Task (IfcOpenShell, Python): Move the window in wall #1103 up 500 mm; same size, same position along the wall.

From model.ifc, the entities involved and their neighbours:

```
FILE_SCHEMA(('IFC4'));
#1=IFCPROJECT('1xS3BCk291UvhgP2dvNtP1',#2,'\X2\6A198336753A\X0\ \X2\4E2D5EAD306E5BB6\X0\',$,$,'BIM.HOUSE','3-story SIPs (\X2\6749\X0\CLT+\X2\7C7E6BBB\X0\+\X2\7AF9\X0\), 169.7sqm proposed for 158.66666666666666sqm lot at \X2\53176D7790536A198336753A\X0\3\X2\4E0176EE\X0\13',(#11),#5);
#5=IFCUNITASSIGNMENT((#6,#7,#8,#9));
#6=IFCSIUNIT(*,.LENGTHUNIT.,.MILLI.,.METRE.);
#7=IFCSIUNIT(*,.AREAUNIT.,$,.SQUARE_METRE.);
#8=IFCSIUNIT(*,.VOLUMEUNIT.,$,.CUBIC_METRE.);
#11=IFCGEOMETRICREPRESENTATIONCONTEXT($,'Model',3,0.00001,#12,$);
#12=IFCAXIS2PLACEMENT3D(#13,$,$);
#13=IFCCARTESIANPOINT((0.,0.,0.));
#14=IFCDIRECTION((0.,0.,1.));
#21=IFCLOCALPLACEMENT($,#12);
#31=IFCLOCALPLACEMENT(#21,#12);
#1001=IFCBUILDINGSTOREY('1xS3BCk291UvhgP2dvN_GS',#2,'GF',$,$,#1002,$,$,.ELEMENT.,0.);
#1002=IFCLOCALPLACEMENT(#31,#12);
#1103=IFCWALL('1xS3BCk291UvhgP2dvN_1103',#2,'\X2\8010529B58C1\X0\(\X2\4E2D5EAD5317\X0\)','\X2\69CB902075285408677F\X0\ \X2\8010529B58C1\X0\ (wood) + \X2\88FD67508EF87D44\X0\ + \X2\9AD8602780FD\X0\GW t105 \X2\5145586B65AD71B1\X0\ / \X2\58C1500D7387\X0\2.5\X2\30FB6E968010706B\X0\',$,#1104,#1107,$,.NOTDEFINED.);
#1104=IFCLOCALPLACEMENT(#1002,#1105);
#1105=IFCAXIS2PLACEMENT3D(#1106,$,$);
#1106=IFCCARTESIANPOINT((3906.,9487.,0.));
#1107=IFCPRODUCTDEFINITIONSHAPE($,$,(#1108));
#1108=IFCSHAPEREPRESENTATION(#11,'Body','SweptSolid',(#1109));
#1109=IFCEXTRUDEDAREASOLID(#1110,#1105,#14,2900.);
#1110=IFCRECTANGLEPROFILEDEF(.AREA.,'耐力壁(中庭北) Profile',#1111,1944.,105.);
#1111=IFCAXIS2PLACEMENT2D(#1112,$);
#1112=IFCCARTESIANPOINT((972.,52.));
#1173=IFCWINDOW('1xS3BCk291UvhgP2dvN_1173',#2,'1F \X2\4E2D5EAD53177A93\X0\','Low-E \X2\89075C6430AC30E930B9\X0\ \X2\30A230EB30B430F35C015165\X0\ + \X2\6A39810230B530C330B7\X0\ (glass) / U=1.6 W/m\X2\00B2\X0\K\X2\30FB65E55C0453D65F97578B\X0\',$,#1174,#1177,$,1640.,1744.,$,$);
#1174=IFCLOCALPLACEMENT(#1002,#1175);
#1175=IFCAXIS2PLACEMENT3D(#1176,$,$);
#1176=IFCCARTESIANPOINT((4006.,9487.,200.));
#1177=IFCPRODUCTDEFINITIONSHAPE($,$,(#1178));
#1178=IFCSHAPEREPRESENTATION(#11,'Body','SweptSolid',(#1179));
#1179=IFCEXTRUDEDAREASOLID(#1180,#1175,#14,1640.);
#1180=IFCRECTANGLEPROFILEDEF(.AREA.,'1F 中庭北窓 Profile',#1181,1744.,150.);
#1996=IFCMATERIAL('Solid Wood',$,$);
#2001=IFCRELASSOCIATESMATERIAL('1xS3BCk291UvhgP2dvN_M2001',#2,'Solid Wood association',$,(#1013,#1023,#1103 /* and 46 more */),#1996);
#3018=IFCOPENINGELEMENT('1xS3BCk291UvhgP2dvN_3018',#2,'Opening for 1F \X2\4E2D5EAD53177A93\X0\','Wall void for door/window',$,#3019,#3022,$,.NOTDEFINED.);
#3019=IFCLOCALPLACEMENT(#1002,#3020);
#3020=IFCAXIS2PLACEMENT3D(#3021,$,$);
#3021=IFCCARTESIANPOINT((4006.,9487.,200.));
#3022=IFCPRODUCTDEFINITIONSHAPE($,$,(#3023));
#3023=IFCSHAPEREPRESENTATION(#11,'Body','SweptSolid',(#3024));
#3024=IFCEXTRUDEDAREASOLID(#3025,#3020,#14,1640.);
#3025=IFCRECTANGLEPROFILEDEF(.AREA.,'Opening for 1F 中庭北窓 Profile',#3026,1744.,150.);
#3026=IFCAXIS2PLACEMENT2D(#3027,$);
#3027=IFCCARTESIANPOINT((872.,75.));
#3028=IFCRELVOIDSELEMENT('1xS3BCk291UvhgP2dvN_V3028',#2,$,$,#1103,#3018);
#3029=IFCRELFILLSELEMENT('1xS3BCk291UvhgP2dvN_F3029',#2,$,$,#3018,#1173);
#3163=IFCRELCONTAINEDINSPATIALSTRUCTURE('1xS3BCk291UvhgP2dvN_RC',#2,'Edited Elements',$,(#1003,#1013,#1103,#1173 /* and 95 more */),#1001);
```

```python
import numpy as np
import ifcopenshell
import ifcopenshell.api.geometry
import ifcopenshell.util.placement
import ifcopenshell.util.unit

model = ifcopenshell.open("model.ifc")
unit_scale = ifcopenshell.util.unit.calculate_unit_scale(model)

window = model.by_guid("1xS3BCk291UvhgP2dvN_1173")
opening = window.FillsVoids[0].RelatingOpeningElement
dz = 500.0

shift = np.array([0.0, 0.0, dz])
# The window is not placed relative to its opening, so move both.
for product in (opening, window):
    matrix = ifcopenshell.util.placement.get_local_placement(product.ObjectPlacement)
    matrix[:3, 3] += shift
    ifcopenshell.api.geometry.edit_object_placement(model, product=product, matrix=matrix, is_si=False)

print(f"moved by {dz * unit_scale:+.3f} m")

model.write("model_edited.ifc")
```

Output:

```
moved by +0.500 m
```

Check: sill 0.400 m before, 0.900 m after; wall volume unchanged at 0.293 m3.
